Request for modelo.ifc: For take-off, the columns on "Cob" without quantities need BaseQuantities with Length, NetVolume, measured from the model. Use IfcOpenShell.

First a look at what the model holds.

```python
import ifcopenshell
import ifcopenshell.util.element
import ifcopenshell.util.unit

model = ifcopenshell.open("modelo.ifc")
print(model.schema)
for unit_type in ("LENGTHUNIT", "AREAUNIT", "VOLUMEUNIT"):
    print(unit_type, ifcopenshell.util.unit.calculate_unit_scale(model, unit_type))
storey = next(s for s in model.by_type("IfcBuildingStorey") if s.Name == "Cob")
columns = [e for e in ifcopenshell.util.element.get_decomposition(storey) if e.is_a("IfcColumn")]
for e in sorted(columns, key=lambda e: e.id()):
    print(e.id(), e.is_a(), e.Name, list(ifcopenshell.util.element.get_psets(e, qtos_only=True)), sep=" | ")
```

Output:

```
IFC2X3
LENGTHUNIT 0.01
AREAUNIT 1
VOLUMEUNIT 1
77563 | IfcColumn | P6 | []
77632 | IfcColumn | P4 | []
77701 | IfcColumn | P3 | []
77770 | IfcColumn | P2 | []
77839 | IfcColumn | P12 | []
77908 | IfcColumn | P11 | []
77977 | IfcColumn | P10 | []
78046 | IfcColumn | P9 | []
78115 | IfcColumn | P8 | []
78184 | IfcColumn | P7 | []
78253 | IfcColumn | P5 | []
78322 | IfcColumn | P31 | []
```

```python
import ifcopenshell
import ifcopenshell.api.pset
import ifcopenshell.geom
import ifcopenshell.util.element
import ifcopenshell.util.shape
import ifcopenshell.util.unit

model = ifcopenshell.open("modelo.ifc")
unit_scale = ifcopenshell.util.unit.calculate_unit_scale(model)
volume_scale = ifcopenshell.util.unit.calculate_unit_scale(model, "VOLUMEUNIT")
settings = ifcopenshell.geom.settings()

storey = next(s for s in model.by_type("IfcBuildingStorey") if s.Name == "Cob")
columns = [e for e in ifcopenshell.util.element.get_decomposition(storey) if e.is_a("IfcColumn")]

for e in sorted(columns, key=lambda e: e.id()):
    if ifcopenshell.util.element.get_psets(e, qtos_only=True, should_inherit=False):
        continue
    # Geometry comes back in metres, in the element's own axes.
    shape = ifcopenshell.geom.create_shape(settings, e)
    values = {
        "Length": ifcopenshell.util.shape.get_z(shape.geometry) / unit_scale,
        "NetVolume": ifcopenshell.util.shape.get_volume(shape.geometry) / volume_scale,
    }
    qto = ifcopenshell.api.pset.add_qto(model, product=e, name="BaseQuantities")
    ifcopenshell.api.pset.edit_qto(model, qto=qto, properties=values)
    print(e.id(), {k: round(v, 3) for k, v in values.items()})

model.write("modelo_rev.ifc")
```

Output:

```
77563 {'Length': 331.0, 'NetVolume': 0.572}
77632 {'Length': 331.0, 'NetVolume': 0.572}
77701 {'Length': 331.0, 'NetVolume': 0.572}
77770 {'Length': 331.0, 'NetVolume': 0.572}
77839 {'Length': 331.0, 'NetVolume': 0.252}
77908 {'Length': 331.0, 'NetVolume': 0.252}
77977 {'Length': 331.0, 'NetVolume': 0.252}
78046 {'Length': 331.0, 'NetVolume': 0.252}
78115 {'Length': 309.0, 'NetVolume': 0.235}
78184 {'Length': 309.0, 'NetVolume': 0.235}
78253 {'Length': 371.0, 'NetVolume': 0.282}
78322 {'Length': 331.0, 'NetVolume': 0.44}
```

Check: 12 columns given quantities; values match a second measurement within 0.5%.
